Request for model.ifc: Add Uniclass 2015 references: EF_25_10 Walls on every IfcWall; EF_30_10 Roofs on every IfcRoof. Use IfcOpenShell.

First a look at what the model holds.

```python
import ifcopenshell

model = ifcopenshell.open("model.ifc")
print(model.schema)
print("classifications:", [c.Name for c in model.by_type("IfcClassification")])
for ifc_class in ("IfcDoor", "IfcRoof", "IfcStair", "IfcWall", "IfcWindow"):
    print(ifc_class, len(model.by_type(ifc_class)))
```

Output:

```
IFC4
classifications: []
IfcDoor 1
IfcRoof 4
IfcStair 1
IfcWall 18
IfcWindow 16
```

```python
import ifcopenshell
import ifcopenshell.api.classification

model = ifcopenshell.open("model.ifc")

system = ifcopenshell.api.classification.add_classification(model, classification="Uniclass 2015")

codes = {
    "IfcWall": ("EF_25_10", "Walls"),
    "IfcRoof": ("EF_30_10", "Roofs"),
}
for ifc_class, (code, name) in codes.items():
    products = model.by_type(ifc_class)
    ifcopenshell.api.classification.add_reference(
        model, products=products, classification=system, identification=code, name=name
    )
    print(code, len(products))

model.write("model_v2.ifc")
```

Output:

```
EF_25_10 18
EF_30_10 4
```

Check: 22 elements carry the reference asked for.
